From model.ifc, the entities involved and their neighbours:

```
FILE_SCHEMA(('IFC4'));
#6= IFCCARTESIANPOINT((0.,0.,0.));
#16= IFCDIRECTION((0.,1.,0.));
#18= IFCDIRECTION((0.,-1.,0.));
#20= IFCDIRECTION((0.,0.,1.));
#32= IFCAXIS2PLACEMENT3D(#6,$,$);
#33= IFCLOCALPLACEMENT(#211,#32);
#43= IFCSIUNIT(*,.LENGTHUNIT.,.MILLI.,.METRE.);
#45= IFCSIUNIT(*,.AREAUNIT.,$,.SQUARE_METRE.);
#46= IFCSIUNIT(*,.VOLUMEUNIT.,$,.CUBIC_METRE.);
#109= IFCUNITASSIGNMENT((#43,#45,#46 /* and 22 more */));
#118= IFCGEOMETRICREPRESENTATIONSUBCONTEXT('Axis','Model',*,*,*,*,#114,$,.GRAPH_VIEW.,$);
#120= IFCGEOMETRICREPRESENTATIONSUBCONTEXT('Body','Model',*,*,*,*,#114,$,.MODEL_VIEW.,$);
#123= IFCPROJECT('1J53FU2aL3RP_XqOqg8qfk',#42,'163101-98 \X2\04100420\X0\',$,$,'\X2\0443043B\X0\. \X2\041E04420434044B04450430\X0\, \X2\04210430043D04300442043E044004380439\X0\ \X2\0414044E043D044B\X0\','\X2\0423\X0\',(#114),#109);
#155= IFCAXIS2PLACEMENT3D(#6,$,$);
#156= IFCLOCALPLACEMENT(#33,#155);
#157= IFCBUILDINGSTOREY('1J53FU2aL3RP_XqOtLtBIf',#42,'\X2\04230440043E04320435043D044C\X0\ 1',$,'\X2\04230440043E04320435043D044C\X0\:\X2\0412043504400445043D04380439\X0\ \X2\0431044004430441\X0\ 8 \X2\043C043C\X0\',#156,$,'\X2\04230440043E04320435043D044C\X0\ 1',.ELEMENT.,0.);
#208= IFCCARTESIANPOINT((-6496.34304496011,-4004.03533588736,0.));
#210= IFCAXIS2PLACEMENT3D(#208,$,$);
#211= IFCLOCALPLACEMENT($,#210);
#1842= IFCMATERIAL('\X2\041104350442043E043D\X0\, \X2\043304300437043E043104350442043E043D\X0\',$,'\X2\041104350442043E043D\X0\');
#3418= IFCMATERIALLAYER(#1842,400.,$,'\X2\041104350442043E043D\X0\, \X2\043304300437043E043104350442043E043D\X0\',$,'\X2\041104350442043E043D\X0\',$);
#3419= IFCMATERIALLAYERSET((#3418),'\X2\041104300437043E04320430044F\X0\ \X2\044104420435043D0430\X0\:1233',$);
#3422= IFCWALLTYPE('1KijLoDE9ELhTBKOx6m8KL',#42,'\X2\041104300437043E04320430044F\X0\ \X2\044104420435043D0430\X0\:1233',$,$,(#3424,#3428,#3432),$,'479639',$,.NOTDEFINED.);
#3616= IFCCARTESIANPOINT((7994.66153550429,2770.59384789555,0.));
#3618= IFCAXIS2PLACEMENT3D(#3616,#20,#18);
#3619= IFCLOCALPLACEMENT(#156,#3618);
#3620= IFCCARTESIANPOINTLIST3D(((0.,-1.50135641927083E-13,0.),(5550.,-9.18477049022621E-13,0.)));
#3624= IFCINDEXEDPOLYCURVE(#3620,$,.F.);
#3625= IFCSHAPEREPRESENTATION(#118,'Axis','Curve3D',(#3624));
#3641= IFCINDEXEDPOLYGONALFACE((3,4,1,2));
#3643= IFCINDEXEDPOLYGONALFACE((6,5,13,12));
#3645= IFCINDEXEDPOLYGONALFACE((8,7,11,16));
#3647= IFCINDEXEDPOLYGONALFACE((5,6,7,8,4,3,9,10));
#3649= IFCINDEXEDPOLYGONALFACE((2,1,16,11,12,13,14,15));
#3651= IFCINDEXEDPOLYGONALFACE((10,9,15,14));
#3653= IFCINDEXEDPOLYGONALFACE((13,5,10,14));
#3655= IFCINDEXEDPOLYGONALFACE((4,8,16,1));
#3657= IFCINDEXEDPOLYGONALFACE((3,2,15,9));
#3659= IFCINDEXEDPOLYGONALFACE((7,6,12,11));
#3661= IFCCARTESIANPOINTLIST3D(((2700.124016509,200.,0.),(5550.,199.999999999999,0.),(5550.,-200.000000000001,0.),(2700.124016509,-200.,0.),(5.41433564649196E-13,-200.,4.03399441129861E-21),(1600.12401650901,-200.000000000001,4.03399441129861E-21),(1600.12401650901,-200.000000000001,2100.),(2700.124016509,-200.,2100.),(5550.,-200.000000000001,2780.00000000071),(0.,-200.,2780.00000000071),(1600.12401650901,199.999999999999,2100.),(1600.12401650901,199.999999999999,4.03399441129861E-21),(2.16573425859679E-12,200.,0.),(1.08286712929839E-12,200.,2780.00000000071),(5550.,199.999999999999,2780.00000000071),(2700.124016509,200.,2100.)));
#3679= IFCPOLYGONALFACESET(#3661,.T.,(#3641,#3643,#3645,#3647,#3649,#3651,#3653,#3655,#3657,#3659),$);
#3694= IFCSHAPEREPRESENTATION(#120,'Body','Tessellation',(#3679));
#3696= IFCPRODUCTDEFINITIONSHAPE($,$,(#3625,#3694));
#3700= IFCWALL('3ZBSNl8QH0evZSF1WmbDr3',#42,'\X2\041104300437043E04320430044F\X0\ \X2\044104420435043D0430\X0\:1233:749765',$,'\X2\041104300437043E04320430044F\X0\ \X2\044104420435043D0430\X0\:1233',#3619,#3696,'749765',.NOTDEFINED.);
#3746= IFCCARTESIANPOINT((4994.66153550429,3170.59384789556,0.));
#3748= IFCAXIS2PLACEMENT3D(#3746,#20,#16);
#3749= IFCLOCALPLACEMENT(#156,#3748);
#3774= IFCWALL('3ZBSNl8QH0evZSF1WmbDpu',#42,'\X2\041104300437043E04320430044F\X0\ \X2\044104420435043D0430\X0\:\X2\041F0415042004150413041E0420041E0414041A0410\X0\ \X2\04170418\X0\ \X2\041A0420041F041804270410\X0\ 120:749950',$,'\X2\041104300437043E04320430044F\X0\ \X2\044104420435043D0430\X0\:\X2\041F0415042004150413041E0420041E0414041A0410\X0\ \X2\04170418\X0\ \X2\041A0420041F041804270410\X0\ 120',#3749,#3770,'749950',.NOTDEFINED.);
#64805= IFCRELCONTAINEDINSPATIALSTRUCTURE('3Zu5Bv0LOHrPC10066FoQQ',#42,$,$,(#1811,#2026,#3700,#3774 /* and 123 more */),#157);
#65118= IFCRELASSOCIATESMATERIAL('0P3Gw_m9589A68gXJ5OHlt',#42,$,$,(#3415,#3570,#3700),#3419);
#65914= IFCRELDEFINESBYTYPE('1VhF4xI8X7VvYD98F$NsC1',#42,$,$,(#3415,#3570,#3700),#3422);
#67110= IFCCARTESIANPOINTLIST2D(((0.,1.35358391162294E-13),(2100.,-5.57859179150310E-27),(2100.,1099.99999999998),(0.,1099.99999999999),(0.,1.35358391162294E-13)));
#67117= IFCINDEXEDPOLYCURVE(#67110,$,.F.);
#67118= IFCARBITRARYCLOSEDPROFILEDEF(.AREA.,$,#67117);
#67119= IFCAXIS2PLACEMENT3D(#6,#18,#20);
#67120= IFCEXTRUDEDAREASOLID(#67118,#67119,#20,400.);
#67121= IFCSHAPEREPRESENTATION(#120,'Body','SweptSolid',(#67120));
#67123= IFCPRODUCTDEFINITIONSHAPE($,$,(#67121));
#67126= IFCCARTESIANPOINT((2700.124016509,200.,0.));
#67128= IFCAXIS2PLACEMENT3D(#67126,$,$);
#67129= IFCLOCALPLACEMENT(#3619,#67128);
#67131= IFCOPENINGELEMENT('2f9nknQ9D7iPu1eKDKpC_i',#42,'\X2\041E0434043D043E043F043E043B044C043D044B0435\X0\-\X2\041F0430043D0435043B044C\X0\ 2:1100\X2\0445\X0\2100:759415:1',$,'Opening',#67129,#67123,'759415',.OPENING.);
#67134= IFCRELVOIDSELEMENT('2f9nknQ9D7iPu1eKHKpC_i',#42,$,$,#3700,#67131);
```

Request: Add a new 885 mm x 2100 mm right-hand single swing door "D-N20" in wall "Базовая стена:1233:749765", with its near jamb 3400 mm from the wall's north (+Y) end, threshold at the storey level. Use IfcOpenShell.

```python
import numpy as np
import ifcopenshell
import ifcopenshell.api.feature
import ifcopenshell.api.geometry
import ifcopenshell.api.root
import ifcopenshell.api.spatial
import ifcopenshell.geom
import ifcopenshell.util.element
import ifcopenshell.util.placement
import ifcopenshell.util.representation
import ifcopenshell.util.shape
import ifcopenshell.util.unit

model = ifcopenshell.open("model.ifc")
unit_scale = ifcopenshell.util.unit.calculate_unit_scale(model)
settings = ifcopenshell.geom.settings()


def volume(element):
    """Net volume in cubic metres, openings subtracted."""
    shape = ifcopenshell.geom.create_shape(settings, element)
    return ifcopenshell.util.shape.get_volume(shape.geometry)


wall = model.by_id(3700)
storey = ifcopenshell.util.element.get_container(wall, ifc_class="IfcBuildingStorey")
context = ifcopenshell.util.representation.get_context(model, "Model", "Body", "MODEL_VIEW")
before = volume(wall)

width, height, from_end, sill = 0.885, 2.1, 3.4, 0.0  # metres

# The wall runs along its own X axis, and the end named is its -X end.
wall_shape = ifcopenshell.geom.create_shape(settings, wall)
x, y, z = ifcopenshell.util.shape.get_vertices(wall_shape.geometry).T
start = x.min() + from_end
face, thickness = float(y.min()), float(y.max() - y.min())
wall_matrix = ifcopenshell.util.placement.get_local_placement(wall.ObjectPlacement)
level = ifcopenshell.util.placement.get_local_placement(storey.ObjectPlacement)[2, 3]


def in_wall(x, y):
    """Placement at x, y metres in the wall's axes, at sill height."""
    matrix = wall_matrix.copy()
    matrix[:, 3] = wall_matrix @ np.array([x / unit_scale, y / unit_scale, 0.0, 1.0])
    matrix[2, 3] = level + sill / unit_scale
    return matrix


# Opening: a box that overshoots both wall faces by 50 mm.
opening = ifcopenshell.api.root.create_entity(model, ifc_class="IfcOpeningElement", predefined_type="OPENING")
box = ifcopenshell.api.geometry.add_wall_representation(
    model, context=context, length=width, height=height, thickness=thickness + 0.1
)
ifcopenshell.api.geometry.assign_representation(model, product=opening, representation=box)
ifcopenshell.api.geometry.edit_object_placement(model, product=opening, matrix=in_wall(start, face - 0.05), is_si=False)
ifcopenshell.api.feature.add_feature(model, feature=opening, element=wall)

door = ifcopenshell.api.root.create_entity(model, ifc_class="IfcDoor", name="D-N20", predefined_type="DOOR")
door.OverallWidth, door.OverallHeight = width / unit_scale, height / unit_scale
door.OperationType = "SINGLE_SWING_RIGHT"
body = ifcopenshell.api.geometry.add_door_representation(
    model,
    context=context,
    overall_width=door.OverallWidth,
    overall_height=door.OverallHeight,
    operation_type="SINGLE_SWING_RIGHT",
    lining_properties={"LiningDepth": thickness / unit_scale, "ThresholdDepth": thickness / unit_scale},
)
ifcopenshell.api.geometry.assign_representation(model, product=door, representation=body)
ifcopenshell.api.spatial.assign_container(model, products=[door], relating_structure=storey)
ifcopenshell.api.feature.add_filling(model, opening=opening, element=door)

# The lining spans the wall, so the door starts at the wall face.
ifcopenshell.api.geometry.edit_object_placement(model, product=door, matrix=in_wall(start, face), is_si=False)

after = volume(wall)

print(f"wall volume {before:.3f} -> {after:.3f} m3")

model.write("model_updated.ifc")
```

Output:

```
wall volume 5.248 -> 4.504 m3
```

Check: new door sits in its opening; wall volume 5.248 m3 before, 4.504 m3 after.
